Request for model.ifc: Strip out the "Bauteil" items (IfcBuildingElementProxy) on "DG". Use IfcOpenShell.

First a look at what the model holds.

```python
import ifcopenshell
import ifcopenshell.util.element

model = ifcopenshell.open("model.ifc")
print(model.schema)
storey = next(s for s in model.by_type("IfcBuildingStorey") if s.Name == "DG")
proxies = [e for e in ifcopenshell.util.element.get_decomposition(storey) if e.is_a("IfcBuildingElementProxy")]
seen = {}
for e in proxies:
    element_type = ifcopenshell.util.element.get_type(e)
    name = element_type.Name if element_type not in (None, e) else None
    seen[name] = seen.get(name, 0) + 1
for name, count in sorted(seen.items(), key=str):
    print(count, "x", name)
```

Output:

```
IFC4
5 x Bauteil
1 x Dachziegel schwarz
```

```python
import ifcopenshell
import ifcopenshell.api.root
import ifcopenshell.util.element

model = ifcopenshell.open("model.ifc")

storey = next(s for s in model.by_type("IfcBuildingStorey") if s.Name == "DG")
proxies = [e for e in ifcopenshell.util.element.get_decomposition(storey) if e.is_a("IfcBuildingElementProxy")]
targets = [e for e in proxies if (t := ifcopenshell.util.element.get_type(e)) not in (None, e) and t.Name == "Bauteil"]

for e in targets:
    ifcopenshell.api.root.remove_product(model, product=e)
print(len(targets), "removed")

model.write("model_v2.ifc")
```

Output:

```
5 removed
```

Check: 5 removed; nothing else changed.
